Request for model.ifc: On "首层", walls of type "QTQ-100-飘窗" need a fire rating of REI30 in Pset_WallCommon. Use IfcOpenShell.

First a look at what the model holds.

```python
import ifcopenshell
import ifcopenshell.util.element

model = ifcopenshell.open("model.ifc")
print(model.schema)
storey = next(s for s in model.by_type("IfcBuildingStorey") if s.Name == "首层")
walls = [e for e in ifcopenshell.util.element.get_decomposition(storey) if e.is_a("IfcWall")]
seen = {}
for e in walls:
    element_type = ifcopenshell.util.element.get_type(e)
    key = (element_type.Name if element_type != e and element_type else None, ifcopenshell.util.element.get_pset(e, "Pset_WallCommon", "FireRating"))
    seen[key] = seen.get(key, 0) + 1
for (name, value), count in sorted(seen.items(), key=str):
    print(count, "x", name, "|", value)
```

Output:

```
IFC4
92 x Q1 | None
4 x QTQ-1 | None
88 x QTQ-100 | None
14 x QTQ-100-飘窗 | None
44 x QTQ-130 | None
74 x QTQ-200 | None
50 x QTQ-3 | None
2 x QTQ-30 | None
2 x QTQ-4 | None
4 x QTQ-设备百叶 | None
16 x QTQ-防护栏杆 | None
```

```python
import ifcopenshell
import ifcopenshell.api.pset
import ifcopenshell.util.element

model = ifcopenshell.open("model.ifc")

storey = next(s for s in model.by_type("IfcBuildingStorey") if s.Name == "首层")
walls = [e for e in ifcopenshell.util.element.get_decomposition(storey) if e.is_a("IfcWall")]

count = 0
for e in walls:
    element_type = ifcopenshell.util.element.get_type(e)
    if element_type in (None, e) or element_type.Name != "QTQ-100-飘窗":
        continue
    # add_pset returns the element's existing set when there is one.
    pset = ifcopenshell.api.pset.add_pset(model, product=e, name="Pset_WallCommon")
    ifcopenshell.api.pset.edit_pset(model, pset=pset, properties={"FireRating": "REI30"})
    count += 1

print(count, "walls updated")

model.write("model_rev.ifc")
```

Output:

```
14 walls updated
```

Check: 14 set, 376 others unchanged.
